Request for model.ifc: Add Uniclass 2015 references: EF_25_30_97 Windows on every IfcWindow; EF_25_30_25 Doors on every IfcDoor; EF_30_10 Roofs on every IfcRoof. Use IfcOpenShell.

First a look at what the model holds.

```python
import ifcopenshell

model = ifcopenshell.open("model.ifc")
print(model.schema)
print("classifications:", [c.Name for c in model.by_type("IfcClassification")])
for ifc_class in ("IfcDoor", "IfcRoof", "IfcStair", "IfcWall", "IfcWindow"):
    print(ifc_class, len(model.by_type(ifc_class)))
```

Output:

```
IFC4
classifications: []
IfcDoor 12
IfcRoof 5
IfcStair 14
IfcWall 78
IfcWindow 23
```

```python
import ifcopenshell
import ifcopenshell.api.classification

model = ifcopenshell.open("model.ifc")

system = ifcopenshell.api.classification.add_classification(model, classification="Uniclass 2015")

codes = {
    "IfcWindow": ("EF_25_30_97", "Windows"),
    "IfcDoor": ("EF_25_30_25", "Doors"),
    "IfcRoof": ("EF_30_10", "Roofs"),
}
for ifc_class, (code, name) in codes.items():
    products = model.by_type(ifc_class)
    ifcopenshell.api.classification.add_reference(
        model, products=products, classification=system, identification=code, name=name
    )
    print(code, len(products))

model.write("model_v2.ifc")
```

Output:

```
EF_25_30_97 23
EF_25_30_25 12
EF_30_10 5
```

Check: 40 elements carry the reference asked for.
